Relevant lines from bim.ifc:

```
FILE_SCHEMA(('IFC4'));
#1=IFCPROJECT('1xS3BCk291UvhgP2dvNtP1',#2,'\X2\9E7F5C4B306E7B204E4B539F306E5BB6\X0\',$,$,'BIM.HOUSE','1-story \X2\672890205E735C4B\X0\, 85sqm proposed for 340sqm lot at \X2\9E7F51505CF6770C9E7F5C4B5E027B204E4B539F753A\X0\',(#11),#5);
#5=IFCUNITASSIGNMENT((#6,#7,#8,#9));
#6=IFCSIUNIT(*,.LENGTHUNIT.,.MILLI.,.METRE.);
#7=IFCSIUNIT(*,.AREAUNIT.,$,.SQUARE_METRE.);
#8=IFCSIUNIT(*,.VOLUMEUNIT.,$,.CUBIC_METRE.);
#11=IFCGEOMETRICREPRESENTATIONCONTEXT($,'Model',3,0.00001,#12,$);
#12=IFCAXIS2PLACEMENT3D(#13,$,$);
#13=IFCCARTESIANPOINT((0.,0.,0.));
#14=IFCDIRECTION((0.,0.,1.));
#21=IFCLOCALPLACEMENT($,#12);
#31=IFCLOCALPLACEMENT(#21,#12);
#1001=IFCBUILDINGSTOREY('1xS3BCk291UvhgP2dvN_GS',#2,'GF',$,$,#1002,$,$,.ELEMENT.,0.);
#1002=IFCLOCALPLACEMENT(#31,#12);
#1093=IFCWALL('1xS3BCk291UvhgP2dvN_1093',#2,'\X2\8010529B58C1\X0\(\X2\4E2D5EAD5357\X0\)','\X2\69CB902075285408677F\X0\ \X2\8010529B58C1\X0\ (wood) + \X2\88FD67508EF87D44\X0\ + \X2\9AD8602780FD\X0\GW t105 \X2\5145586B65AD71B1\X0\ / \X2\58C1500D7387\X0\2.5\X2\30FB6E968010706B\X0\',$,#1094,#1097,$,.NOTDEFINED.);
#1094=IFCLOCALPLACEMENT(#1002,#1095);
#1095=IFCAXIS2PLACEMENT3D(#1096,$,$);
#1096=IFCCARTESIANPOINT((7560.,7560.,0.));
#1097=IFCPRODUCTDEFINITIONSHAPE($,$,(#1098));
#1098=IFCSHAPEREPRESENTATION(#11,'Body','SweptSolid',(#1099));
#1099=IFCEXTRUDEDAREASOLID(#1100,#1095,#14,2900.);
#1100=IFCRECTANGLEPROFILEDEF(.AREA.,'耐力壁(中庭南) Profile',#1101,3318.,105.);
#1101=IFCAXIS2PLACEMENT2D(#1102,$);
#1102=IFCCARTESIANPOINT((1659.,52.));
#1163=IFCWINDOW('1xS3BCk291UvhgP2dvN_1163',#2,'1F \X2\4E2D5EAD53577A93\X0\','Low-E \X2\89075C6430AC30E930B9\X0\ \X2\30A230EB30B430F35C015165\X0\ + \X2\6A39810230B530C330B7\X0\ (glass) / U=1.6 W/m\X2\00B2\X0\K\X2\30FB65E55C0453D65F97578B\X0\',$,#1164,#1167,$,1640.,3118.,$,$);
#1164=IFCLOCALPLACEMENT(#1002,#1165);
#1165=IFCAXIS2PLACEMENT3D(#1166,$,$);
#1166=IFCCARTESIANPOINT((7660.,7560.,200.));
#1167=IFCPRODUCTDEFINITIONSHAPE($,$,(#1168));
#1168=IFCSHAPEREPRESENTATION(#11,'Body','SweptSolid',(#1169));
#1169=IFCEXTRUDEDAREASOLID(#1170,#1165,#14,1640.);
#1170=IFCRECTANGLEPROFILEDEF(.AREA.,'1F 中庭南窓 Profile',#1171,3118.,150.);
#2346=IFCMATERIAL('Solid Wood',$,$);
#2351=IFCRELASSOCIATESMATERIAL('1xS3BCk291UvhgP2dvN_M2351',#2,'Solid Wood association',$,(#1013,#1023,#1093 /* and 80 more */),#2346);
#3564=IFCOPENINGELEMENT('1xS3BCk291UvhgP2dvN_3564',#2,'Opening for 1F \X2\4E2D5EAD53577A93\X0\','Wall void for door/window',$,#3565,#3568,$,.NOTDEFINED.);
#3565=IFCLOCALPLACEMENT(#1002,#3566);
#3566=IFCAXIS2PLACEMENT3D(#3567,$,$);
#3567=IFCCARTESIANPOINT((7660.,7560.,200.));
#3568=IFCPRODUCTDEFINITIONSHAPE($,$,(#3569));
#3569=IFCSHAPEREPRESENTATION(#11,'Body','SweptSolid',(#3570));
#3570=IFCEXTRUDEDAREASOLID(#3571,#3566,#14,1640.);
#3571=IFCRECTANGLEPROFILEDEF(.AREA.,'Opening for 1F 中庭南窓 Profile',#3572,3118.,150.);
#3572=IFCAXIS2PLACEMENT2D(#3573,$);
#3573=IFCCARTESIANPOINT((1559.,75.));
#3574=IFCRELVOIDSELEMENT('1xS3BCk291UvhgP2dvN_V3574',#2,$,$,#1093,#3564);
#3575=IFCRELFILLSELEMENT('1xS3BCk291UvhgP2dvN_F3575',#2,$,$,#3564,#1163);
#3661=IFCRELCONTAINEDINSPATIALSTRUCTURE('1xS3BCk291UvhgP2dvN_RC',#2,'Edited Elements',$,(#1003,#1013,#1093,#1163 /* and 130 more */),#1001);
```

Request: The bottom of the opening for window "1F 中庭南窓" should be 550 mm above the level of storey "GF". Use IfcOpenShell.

```python
import numpy as np
import ifcopenshell
import ifcopenshell.api.geometry
import ifcopenshell.geom
import ifcopenshell.util.element
import ifcopenshell.util.placement
import ifcopenshell.util.shape
import ifcopenshell.util.unit

model = ifcopenshell.open("bim.ifc")
unit_scale = ifcopenshell.util.unit.calculate_unit_scale(model)

window = model.by_id(1163)
opening = window.FillsVoids[0].RelatingOpeningElement
storey = ifcopenshell.util.element.get_container(window, ifc_class="IfcBuildingStorey")
level = ifcopenshell.util.placement.get_local_placement(storey.ObjectPlacement)[2, 3]

# The opening's origin need not be at the sill, so measure its lowest point.
shape = ifcopenshell.geom.create_shape(ifcopenshell.geom.settings(), opening)
bottom = ifcopenshell.util.shape.get_shape_bottom_elevation(shape, shape.geometry) / unit_scale
dz = level + 0.55 / unit_scale - bottom

shift = np.array([0.0, 0.0, dz])
# The window is not placed relative to its opening, so move both.
for product in (opening, window):
    matrix = ifcopenshell.util.placement.get_local_placement(product.ObjectPlacement)
    matrix[:3, 3] += shift
    ifcopenshell.api.geometry.edit_object_placement(model, product=product, matrix=matrix, is_si=False)

print(f"moved by {dz * unit_scale:+.3f} m")

model.write("bim_edited.ifc")
```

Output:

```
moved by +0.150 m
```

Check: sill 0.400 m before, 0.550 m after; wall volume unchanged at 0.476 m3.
